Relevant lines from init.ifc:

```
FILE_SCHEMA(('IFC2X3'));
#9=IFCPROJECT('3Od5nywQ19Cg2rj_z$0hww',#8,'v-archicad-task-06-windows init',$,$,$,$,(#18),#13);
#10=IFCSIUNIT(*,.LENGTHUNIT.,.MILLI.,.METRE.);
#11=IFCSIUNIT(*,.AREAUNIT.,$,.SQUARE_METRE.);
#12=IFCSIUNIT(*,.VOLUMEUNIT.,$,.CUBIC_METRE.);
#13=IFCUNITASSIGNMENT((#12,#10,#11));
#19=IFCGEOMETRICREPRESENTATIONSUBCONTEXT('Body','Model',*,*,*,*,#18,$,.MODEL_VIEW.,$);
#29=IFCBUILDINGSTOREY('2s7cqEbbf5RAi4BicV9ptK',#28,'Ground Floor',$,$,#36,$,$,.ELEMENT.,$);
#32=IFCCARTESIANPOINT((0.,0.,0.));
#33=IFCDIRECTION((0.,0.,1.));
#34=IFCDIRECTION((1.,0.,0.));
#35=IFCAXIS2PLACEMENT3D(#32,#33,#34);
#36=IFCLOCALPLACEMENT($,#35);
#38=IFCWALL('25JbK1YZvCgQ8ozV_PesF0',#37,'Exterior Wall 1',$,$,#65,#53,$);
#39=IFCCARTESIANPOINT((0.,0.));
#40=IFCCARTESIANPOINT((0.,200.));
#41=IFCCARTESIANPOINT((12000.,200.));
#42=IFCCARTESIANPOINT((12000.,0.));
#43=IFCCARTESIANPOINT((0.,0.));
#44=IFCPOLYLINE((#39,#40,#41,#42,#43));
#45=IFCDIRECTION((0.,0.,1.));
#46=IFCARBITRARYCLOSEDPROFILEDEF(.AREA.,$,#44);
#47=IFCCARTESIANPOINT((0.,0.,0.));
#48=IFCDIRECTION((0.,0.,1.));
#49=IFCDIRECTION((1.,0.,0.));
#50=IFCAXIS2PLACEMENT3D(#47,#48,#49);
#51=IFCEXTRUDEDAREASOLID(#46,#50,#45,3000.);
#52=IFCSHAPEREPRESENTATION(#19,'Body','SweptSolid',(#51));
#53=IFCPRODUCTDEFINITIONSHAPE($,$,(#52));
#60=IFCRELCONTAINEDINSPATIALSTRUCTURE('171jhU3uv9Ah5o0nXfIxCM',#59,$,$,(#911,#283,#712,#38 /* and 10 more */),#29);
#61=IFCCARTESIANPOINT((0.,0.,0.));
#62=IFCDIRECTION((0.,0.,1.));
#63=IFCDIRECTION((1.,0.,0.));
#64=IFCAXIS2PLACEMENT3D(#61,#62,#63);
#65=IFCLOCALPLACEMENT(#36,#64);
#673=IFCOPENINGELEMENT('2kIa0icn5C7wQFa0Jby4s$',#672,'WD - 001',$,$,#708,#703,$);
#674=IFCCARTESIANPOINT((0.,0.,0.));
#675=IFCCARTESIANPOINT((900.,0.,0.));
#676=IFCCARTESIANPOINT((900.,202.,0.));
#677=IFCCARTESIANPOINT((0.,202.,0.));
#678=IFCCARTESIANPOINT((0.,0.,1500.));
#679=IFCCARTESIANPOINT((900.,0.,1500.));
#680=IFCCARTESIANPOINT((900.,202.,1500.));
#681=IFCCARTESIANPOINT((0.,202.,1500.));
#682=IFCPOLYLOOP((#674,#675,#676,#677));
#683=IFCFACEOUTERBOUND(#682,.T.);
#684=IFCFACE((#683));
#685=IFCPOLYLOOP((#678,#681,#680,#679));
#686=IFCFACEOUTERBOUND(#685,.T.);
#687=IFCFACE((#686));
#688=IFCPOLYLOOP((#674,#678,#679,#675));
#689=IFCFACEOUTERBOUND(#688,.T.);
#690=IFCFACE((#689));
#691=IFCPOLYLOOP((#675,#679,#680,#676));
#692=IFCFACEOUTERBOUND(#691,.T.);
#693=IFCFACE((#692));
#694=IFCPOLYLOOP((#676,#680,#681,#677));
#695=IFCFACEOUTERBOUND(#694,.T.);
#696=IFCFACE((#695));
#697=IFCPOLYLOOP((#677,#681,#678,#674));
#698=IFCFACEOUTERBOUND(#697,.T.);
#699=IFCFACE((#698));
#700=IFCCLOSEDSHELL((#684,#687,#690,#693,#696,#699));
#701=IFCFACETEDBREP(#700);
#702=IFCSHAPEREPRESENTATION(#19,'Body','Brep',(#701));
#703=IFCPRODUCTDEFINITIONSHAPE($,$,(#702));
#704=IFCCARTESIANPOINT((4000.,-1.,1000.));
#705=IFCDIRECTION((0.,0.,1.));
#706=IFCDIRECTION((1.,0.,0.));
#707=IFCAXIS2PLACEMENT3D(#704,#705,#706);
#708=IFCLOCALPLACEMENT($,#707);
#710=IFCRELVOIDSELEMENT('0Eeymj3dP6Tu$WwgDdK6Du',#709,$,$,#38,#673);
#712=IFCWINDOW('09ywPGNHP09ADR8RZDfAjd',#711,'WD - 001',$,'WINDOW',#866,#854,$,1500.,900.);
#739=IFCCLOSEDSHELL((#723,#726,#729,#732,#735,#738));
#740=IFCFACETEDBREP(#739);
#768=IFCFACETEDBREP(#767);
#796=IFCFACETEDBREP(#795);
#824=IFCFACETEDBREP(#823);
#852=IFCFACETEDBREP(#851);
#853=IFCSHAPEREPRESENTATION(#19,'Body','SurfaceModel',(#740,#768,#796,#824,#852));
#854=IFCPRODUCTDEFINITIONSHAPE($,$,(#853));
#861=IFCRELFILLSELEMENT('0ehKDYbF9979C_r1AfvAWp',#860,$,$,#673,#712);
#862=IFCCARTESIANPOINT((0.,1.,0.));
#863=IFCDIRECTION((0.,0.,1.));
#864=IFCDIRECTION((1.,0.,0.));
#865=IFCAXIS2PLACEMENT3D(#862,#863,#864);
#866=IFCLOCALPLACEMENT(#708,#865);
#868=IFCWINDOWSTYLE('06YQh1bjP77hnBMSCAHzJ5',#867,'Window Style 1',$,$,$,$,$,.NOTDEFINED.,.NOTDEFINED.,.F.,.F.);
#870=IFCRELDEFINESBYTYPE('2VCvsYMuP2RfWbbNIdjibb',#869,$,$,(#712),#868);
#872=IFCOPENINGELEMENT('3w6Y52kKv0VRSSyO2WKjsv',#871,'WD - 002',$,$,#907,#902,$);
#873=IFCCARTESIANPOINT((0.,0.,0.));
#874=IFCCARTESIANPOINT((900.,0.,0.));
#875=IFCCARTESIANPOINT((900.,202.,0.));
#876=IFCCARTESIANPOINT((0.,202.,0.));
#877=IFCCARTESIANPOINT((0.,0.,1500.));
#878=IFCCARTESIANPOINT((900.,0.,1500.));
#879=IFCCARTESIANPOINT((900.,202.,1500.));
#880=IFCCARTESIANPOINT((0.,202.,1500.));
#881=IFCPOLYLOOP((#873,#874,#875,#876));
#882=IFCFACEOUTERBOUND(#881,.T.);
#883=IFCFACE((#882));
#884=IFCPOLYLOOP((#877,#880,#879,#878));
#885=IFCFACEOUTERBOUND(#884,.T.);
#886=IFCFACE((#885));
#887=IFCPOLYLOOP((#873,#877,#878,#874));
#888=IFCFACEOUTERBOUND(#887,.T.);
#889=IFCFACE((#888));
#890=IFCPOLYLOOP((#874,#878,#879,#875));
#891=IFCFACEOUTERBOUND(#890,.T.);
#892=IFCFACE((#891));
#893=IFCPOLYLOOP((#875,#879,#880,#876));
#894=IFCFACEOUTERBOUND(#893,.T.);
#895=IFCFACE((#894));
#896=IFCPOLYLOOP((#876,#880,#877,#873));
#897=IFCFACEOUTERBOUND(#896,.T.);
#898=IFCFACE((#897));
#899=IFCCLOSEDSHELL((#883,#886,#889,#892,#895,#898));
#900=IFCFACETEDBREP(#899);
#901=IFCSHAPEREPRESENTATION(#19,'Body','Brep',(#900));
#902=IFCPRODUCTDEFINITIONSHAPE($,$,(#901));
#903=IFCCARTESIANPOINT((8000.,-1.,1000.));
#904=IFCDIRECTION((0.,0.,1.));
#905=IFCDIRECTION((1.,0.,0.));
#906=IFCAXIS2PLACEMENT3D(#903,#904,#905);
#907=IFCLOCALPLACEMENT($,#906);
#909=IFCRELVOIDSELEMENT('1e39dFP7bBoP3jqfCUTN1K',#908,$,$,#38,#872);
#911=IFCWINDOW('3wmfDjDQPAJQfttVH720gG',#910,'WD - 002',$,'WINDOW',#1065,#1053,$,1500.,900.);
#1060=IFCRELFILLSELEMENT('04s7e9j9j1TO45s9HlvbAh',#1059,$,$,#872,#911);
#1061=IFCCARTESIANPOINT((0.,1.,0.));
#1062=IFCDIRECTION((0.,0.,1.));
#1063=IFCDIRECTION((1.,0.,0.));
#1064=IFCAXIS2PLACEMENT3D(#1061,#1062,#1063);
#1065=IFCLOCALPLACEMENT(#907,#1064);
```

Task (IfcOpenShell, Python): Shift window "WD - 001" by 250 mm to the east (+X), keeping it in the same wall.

```python
import ifcopenshell
import ifcopenshell.api.geometry
import ifcopenshell.util.placement
import ifcopenshell.util.unit

model = ifcopenshell.open("init.ifc")
unit_scale = ifcopenshell.util.unit.calculate_unit_scale(model)

window = model.by_guid("09ywPGNHP09ADR8RZDfAjd")
opening = window.FillsVoids[0].RelatingOpeningElement
wall = opening.VoidsElements[0].RelatingBuildingElement

wall_matrix = ifcopenshell.util.placement.get_local_placement(wall.ObjectPlacement)
shift = wall_matrix[:3, 0] * 0.25 / unit_scale
before = ifcopenshell.util.placement.get_local_placement(window.ObjectPlacement)[:3, 3].copy()

# The window is placed relative to its opening, so it follows when the opening moves.
matrix = ifcopenshell.util.placement.get_local_placement(opening.ObjectPlacement)
matrix[:3, 3] += shift
ifcopenshell.api.geometry.edit_object_placement(
    model, product=opening, matrix=matrix, is_si=False, should_transform_children=True
)

after = ifcopenshell.util.placement.get_local_placement(window.ObjectPlacement)[:3, 3]
print("window moved by", (after - before).round(3) + 0.0)

model.write("init_v2.ifc")
```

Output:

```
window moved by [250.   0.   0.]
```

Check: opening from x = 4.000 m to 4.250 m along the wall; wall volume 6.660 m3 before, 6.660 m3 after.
